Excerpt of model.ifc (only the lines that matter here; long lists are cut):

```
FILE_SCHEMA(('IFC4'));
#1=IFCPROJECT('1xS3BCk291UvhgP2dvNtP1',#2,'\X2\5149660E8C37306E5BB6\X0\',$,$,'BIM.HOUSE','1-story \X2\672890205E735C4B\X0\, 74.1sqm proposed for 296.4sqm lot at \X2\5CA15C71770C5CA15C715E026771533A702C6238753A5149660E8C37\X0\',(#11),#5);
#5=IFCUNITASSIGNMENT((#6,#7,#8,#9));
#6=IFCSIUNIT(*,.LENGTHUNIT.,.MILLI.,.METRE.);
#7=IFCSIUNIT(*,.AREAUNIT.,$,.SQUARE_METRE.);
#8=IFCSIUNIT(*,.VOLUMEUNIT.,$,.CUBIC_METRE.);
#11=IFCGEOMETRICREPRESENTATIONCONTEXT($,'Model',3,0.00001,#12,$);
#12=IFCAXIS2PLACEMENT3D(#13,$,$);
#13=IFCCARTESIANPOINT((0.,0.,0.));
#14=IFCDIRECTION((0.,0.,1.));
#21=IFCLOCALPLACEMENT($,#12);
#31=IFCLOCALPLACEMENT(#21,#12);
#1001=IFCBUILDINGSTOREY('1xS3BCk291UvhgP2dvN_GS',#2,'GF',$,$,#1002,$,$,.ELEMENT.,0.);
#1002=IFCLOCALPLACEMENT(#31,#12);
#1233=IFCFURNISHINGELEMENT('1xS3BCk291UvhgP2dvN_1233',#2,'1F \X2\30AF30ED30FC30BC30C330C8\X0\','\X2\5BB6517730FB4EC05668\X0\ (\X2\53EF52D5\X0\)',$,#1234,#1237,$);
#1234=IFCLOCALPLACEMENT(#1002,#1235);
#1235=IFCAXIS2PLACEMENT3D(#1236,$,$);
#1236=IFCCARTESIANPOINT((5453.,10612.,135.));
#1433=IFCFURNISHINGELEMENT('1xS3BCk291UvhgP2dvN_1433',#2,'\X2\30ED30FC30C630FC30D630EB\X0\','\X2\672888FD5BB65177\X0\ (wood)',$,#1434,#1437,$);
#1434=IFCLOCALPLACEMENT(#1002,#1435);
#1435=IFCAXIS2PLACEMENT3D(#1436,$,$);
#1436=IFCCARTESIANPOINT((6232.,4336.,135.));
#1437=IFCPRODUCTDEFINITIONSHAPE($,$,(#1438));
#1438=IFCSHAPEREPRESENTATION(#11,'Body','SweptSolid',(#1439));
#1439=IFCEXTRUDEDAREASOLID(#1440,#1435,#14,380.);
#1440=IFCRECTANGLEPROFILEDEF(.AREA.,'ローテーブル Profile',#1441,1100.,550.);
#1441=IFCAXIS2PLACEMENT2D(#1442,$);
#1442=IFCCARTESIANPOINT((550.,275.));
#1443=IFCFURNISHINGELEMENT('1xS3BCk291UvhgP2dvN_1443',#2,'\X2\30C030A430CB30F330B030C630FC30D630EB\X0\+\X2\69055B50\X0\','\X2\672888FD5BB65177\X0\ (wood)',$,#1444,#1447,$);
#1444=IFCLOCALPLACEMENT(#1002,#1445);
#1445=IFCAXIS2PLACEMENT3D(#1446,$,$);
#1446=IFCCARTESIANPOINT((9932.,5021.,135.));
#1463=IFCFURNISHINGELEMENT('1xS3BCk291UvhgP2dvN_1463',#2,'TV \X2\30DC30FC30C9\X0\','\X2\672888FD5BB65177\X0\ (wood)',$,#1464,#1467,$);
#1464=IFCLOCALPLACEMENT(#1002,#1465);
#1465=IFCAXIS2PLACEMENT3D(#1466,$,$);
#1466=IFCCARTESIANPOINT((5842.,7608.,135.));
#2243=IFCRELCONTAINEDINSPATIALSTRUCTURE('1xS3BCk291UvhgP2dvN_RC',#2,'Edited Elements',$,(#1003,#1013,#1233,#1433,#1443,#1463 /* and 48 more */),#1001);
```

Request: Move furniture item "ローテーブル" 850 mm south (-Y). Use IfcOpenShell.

```python
import ifcopenshell
import ifcopenshell.api.geometry
import ifcopenshell.util.placement

model = ifcopenshell.open("model.ifc")

item = model.by_guid("1xS3BCk291UvhgP2dvN_1433")
matrix = ifcopenshell.util.placement.get_local_placement(item.ObjectPlacement)
matrix[1, 3] -= 850.0
ifcopenshell.api.geometry.edit_object_placement(model, product=item, matrix=matrix, is_si=False)

print(ifcopenshell.util.placement.get_local_placement(item.ObjectPlacement).round(3) + 0.0)

model.write("model_edited.ifc")
```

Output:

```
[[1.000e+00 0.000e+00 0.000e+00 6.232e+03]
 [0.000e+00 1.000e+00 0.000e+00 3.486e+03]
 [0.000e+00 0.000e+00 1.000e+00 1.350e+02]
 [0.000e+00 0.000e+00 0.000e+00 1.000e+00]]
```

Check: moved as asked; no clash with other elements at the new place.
